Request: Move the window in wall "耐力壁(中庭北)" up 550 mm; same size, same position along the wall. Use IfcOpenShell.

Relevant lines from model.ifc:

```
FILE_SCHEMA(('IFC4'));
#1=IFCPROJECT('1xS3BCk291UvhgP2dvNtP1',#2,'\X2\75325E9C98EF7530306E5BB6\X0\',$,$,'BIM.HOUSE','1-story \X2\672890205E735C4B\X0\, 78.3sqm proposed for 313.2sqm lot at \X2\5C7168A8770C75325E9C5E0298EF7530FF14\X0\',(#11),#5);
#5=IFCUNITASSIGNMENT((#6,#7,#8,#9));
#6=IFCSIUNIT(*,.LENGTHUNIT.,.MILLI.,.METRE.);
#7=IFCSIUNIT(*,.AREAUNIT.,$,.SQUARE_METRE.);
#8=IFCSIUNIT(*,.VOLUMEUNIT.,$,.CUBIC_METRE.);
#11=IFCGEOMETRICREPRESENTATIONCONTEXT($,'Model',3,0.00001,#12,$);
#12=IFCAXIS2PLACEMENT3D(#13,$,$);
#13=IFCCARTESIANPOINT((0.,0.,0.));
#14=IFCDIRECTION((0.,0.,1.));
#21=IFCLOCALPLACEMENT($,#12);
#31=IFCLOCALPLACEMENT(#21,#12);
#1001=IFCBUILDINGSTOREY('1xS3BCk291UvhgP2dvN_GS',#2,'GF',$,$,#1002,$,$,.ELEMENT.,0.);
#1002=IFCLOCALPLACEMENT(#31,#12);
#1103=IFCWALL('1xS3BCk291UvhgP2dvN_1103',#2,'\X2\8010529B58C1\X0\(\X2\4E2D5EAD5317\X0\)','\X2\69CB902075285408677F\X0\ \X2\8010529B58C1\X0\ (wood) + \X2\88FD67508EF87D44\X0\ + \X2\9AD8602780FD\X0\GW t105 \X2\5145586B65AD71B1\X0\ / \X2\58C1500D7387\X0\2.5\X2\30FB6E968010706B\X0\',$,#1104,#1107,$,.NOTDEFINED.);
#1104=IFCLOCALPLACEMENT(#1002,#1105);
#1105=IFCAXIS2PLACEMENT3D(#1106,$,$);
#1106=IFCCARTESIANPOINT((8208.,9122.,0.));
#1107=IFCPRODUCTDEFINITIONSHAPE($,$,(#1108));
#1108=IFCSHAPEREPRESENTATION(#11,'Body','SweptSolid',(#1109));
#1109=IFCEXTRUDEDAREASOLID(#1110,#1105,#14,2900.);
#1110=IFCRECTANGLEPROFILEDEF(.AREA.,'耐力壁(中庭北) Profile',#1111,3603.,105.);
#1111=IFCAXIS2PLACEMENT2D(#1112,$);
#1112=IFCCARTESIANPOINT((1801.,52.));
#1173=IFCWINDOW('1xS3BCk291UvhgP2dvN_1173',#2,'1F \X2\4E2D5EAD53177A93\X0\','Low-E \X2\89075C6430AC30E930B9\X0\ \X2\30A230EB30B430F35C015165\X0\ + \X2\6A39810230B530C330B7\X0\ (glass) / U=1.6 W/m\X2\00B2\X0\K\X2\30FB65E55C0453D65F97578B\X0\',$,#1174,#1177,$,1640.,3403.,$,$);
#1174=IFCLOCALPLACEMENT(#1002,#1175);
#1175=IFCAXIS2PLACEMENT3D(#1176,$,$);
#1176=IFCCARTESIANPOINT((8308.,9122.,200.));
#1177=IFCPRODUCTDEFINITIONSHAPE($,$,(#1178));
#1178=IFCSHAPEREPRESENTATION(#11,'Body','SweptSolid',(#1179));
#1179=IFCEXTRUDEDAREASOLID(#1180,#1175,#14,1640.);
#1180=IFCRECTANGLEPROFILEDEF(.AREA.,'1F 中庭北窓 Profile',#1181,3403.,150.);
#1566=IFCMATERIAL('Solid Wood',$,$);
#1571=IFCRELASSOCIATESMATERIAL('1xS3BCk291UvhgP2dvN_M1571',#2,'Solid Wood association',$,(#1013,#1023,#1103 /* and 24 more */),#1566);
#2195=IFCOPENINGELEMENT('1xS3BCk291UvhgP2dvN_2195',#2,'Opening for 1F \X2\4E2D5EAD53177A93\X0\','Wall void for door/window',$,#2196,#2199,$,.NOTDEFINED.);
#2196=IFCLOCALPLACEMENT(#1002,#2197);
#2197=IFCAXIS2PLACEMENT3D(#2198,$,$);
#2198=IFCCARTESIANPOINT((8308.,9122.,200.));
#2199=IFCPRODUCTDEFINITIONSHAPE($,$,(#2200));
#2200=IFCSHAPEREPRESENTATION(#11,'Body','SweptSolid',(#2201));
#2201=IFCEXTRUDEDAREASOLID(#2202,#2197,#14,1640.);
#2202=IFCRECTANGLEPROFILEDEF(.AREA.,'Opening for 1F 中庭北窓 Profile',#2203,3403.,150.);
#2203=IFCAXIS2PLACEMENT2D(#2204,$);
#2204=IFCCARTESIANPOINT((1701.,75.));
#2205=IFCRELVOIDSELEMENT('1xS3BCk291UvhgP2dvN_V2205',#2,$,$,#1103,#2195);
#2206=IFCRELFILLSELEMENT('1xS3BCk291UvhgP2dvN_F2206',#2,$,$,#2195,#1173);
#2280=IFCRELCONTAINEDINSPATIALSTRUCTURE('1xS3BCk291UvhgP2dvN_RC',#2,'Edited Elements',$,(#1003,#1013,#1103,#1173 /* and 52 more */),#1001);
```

```python
import numpy as np
import ifcopenshell
import ifcopenshell.api.geometry
import ifcopenshell.util.placement
import ifcopenshell.util.unit

model = ifcopenshell.open("model.ifc")
unit_scale = ifcopenshell.util.unit.calculate_unit_scale(model)

window = model.by_id(1173)
opening = window.FillsVoids[0].RelatingOpeningElement
dz = 0.55 / unit_scale

shift = np.array([0.0, 0.0, dz])
# The window is not placed relative to its opening, so move both.
for product in (opening, window):
    matrix = ifcopenshell.util.placement.get_local_placement(product.ObjectPlacement)
    matrix[:3, 3] += shift
    ifcopenshell.api.geometry.edit_object_placement(model, product=product, matrix=matrix, is_si=False)

print(f"moved by {dz * unit_scale:+.3f} m")

model.write("model_v2.ifc")
```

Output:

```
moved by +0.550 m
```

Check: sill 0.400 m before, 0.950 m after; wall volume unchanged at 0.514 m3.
